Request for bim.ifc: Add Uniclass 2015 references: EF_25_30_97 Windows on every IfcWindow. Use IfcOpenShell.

First a look at what the model holds.

```python
import ifcopenshell

model = ifcopenshell.open("bim.ifc")
print(model.schema)
print("classifications:", [c.Name for c in model.by_type("IfcClassification")])
for ifc_class in ("IfcDoor", "IfcRoof", "IfcStair", "IfcWall", "IfcWindow"):
    print(ifc_class, len(model.by_type(ifc_class)))
```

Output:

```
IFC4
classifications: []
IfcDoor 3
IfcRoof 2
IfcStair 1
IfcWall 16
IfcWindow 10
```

```python
import ifcopenshell
import ifcopenshell.api.classification

model = ifcopenshell.open("bim.ifc")

system = ifcopenshell.api.classification.add_classification(model, classification="Uniclass 2015")

codes = {
    "IfcWindow": ("EF_25_30_97", "Windows"),
}
for ifc_class, (code, name) in codes.items():
    products = model.by_type(ifc_class)
    ifcopenshell.api.classification.add_reference(
        model, products=products, classification=system, identification=code, name=name
    )
    print(code, len(products))

model.write("bim_updated.ifc")
```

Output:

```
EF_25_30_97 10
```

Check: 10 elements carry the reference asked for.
